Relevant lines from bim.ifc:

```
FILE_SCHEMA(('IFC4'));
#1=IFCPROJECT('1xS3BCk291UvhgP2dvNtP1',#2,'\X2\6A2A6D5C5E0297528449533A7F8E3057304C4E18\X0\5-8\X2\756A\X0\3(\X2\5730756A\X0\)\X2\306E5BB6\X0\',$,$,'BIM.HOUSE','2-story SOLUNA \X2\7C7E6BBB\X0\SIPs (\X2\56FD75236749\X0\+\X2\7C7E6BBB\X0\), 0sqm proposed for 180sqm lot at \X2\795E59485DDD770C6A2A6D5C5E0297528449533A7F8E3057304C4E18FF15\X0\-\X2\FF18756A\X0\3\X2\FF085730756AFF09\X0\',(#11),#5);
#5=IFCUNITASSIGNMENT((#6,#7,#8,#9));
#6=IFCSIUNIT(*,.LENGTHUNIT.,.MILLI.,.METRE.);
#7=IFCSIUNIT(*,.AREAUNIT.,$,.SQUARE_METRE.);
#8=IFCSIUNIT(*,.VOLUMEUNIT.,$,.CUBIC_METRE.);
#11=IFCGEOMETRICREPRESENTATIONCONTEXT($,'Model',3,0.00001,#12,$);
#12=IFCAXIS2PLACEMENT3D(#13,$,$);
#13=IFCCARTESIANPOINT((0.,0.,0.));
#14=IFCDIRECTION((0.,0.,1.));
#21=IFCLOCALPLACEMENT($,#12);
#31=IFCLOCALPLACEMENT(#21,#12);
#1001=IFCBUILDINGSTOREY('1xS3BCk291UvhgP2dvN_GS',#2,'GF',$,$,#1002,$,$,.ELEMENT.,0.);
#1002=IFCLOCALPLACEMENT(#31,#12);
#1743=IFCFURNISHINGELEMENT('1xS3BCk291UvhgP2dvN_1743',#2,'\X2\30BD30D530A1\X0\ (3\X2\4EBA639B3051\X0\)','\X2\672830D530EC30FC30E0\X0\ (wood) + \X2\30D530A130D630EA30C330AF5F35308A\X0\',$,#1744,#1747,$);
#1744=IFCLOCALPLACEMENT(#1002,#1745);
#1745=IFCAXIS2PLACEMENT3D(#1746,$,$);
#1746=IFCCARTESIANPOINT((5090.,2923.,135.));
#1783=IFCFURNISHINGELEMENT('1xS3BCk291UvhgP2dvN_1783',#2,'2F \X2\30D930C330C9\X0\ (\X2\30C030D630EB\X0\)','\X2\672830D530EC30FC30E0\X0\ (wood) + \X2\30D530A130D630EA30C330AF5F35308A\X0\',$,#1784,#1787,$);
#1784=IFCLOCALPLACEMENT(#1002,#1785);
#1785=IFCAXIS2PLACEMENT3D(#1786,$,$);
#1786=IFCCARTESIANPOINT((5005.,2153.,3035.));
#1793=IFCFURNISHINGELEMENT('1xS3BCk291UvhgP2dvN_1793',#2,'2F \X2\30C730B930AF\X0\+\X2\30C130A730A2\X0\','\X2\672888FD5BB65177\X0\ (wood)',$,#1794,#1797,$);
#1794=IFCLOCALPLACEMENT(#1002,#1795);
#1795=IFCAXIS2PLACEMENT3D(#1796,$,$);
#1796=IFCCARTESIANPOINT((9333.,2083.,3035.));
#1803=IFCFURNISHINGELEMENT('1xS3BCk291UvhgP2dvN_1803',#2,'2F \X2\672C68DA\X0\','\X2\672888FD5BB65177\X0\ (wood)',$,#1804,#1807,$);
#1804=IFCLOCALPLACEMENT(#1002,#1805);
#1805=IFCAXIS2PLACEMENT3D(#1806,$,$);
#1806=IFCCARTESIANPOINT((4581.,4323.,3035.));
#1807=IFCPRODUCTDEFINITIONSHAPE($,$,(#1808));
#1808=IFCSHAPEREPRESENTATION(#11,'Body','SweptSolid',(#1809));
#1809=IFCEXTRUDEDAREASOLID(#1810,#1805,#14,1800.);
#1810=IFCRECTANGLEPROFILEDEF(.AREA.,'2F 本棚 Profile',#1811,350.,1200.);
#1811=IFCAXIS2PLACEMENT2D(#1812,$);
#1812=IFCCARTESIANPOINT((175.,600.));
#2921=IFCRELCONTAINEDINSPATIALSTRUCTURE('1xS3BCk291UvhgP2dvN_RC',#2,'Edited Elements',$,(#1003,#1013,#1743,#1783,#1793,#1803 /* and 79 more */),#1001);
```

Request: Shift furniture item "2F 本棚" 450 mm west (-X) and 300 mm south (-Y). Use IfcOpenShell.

```python
import ifcopenshell
import ifcopenshell.api.geometry
import ifcopenshell.util.placement
import ifcopenshell.util.unit

model = ifcopenshell.open("bim.ifc")
unit_scale = ifcopenshell.util.unit.calculate_unit_scale(model)

item = model.by_id(1803)
matrix = ifcopenshell.util.placement.get_local_placement(item.ObjectPlacement)
matrix[0, 3] -= 0.45 / unit_scale
matrix[1, 3] -= 0.3 / unit_scale
ifcopenshell.api.geometry.edit_object_placement(model, product=item, matrix=matrix, is_si=False)

print(ifcopenshell.util.placement.get_local_placement(item.ObjectPlacement).round(3) + 0.0)

model.write("bim-out.ifc")
```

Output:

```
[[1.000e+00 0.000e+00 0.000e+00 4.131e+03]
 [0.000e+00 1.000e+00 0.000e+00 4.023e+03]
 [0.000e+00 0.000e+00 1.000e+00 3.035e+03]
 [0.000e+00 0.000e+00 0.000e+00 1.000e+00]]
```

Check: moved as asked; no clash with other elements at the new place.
